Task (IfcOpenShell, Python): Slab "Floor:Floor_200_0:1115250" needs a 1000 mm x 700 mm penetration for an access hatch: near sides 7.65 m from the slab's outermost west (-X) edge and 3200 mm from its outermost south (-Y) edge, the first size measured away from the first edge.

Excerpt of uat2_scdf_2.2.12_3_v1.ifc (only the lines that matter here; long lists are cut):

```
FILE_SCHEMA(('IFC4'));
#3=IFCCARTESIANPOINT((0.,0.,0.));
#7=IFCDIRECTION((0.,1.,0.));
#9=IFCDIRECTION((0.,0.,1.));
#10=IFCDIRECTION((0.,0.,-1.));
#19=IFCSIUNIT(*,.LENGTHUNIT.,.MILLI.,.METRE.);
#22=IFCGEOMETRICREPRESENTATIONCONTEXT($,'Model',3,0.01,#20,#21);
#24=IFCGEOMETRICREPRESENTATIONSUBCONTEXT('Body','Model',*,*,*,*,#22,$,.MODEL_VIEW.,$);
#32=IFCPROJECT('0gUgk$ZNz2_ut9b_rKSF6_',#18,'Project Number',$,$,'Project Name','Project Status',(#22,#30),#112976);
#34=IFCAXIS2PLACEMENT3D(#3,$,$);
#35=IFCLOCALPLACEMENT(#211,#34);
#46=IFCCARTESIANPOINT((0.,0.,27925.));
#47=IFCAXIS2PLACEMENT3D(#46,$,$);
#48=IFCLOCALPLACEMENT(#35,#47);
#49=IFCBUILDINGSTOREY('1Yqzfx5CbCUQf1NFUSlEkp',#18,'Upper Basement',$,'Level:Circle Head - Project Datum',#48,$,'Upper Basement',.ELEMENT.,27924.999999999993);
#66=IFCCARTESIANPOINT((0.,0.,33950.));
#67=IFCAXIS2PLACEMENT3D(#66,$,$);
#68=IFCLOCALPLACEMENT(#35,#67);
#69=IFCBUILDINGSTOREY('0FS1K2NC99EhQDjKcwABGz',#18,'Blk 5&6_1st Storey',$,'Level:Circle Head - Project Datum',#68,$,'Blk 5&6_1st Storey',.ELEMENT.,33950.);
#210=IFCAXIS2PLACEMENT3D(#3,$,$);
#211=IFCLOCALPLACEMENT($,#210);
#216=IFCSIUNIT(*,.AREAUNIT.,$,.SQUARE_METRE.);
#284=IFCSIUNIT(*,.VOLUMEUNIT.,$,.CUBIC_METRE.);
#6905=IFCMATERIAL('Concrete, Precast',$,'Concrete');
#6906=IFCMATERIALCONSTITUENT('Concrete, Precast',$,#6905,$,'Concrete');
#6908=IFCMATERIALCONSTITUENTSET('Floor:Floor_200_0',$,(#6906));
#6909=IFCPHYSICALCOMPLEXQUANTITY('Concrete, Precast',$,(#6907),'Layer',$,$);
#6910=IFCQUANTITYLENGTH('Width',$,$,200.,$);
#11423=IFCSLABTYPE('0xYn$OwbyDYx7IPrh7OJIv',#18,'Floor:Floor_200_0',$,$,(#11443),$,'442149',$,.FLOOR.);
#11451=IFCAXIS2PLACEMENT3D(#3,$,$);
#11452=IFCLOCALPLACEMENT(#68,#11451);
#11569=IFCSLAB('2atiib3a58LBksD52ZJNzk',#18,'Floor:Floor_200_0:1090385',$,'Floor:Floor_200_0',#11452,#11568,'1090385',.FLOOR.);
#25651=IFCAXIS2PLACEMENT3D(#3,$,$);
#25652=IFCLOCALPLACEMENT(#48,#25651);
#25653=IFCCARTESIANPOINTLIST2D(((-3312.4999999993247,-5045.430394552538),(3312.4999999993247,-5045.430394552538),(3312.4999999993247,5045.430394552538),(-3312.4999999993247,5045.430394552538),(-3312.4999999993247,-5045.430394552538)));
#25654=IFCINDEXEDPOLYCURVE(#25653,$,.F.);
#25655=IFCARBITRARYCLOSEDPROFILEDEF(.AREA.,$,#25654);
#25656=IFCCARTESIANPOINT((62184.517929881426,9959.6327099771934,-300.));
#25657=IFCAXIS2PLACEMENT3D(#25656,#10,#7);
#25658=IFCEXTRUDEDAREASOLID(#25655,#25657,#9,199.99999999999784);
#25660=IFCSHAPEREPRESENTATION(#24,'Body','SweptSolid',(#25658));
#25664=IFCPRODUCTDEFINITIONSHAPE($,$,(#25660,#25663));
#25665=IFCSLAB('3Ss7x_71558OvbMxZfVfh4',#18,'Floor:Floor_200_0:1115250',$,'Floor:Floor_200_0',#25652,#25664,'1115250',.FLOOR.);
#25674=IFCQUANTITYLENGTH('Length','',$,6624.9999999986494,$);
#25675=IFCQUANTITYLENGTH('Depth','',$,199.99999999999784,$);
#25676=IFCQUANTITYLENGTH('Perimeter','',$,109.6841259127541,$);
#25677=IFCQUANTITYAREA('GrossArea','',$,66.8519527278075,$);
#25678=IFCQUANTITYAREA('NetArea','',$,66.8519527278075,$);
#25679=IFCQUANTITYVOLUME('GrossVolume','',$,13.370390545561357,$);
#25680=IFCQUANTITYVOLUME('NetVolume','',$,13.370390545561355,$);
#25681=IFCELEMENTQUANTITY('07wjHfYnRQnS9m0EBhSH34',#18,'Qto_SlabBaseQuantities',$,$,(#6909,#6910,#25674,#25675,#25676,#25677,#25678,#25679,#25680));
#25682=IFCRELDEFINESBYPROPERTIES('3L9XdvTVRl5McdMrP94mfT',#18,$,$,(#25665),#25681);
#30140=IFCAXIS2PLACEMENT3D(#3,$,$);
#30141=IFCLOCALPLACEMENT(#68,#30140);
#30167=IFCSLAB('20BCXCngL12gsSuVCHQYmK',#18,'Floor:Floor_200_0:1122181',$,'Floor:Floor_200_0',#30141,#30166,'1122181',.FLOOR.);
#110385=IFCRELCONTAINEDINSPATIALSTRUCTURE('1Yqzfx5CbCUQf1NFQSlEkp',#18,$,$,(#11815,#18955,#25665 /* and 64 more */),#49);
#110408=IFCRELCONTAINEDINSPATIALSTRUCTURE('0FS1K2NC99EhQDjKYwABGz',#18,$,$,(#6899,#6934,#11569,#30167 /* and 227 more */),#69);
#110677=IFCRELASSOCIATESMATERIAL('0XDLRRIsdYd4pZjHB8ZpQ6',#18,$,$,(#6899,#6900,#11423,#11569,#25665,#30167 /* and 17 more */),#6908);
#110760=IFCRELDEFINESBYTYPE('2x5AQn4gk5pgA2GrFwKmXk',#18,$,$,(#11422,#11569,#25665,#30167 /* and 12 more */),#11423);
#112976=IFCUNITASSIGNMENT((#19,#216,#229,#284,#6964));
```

```python
import numpy as np
import ifcopenshell
import ifcopenshell.api.feature
import ifcopenshell.api.geometry
import ifcopenshell.api.pset
import ifcopenshell.api.root
import ifcopenshell.geom
import ifcopenshell.util.element
import ifcopenshell.util.placement
import ifcopenshell.util.representation
import ifcopenshell.util.shape
import ifcopenshell.util.unit

model = ifcopenshell.open("uat2_scdf_2.2.12_3_v1.ifc")
unit_scale = ifcopenshell.util.unit.calculate_unit_scale(model)
area_scale = ifcopenshell.util.unit.calculate_unit_scale(model, "AREAUNIT")
volume_scale = ifcopenshell.util.unit.calculate_unit_scale(model, "VOLUMEUNIT")
settings = ifcopenshell.geom.settings()


def volume(element):
    """Net volume in cubic metres, openings subtracted."""
    shape = ifcopenshell.geom.create_shape(settings, element)
    return ifcopenshell.util.shape.get_volume(shape.geometry)


slab = model.by_guid("3Ss7x_71558OvbMxZfVfh4")
before = volume(slab)

# Extent in the slab's own axes, in metres. The edges named are its -X and -Y sides.
slab_shape = ifcopenshell.geom.create_shape(settings, slab)
vertices = ifcopenshell.util.shape.get_vertices(slab_shape.geometry)
x_min, y_min, bottom = vertices.min(axis=0)
top = vertices[:, 2].max()

opening = ifcopenshell.api.root.create_entity(model, ifc_class="IfcOpeningElement", name="Access hatch opening", predefined_type="OPENING")
context = ifcopenshell.util.representation.get_context(model, "Model", "Body", "MODEL_VIEW")
width, depth = 1, 0.7
outline = [(0.0, 0.0), (width, 0.0), (width, depth), (0.0, depth), (0.0, 0.0)]
# Overshoot both faces by 50 mm so the cut is clean.
shape = ifcopenshell.api.geometry.add_slab_representation(
    model, context=context, depth=top - bottom + 0.1, polyline=outline
)
ifcopenshell.api.geometry.assign_representation(model, product=opening, representation=shape)

matrix = ifcopenshell.util.placement.get_local_placement(slab.ObjectPlacement)
matrix[:, 3] = matrix @ np.append(np.array([x_min + 7.65, y_min + 3.2, bottom - 0.05]) / unit_scale, 1.0)
ifcopenshell.api.geometry.edit_object_placement(model, product=opening, matrix=matrix, is_si=False)
ifcopenshell.api.feature.add_feature(model, feature=opening, element=slab)

after = volume(slab)

# Update the slab's stored quantities.
qto = model.by_id(ifcopenshell.util.element.get_pset(slab, "Qto_SlabBaseQuantities", should_inherit=False)["id"])
ifcopenshell.api.pset.edit_qto(model, qto=qto, properties={
    "NetArea": after / (top - bottom) / area_scale,
    "NetVolume": after / volume_scale,
})

print(f"slab volume {before:.3f} -> {after:.3f} m3")

model.write("uat2_scdf_2.2.12_3_v1_v2.ifc")
```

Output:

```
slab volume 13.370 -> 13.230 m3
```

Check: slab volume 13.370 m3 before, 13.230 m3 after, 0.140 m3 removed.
